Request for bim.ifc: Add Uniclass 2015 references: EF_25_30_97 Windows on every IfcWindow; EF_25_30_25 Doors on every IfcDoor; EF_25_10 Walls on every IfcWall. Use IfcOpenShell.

First a look at what the model holds.

```python
import ifcopenshell

model = ifcopenshell.open("bim.ifc")
print(model.schema)
print("classifications:", [c.Name for c in model.by_type("IfcClassification")])
for ifc_class in ("IfcDoor", "IfcRoof", "IfcStair", "IfcWall", "IfcWindow"):
    print(ifc_class, len(model.by_type(ifc_class)))
```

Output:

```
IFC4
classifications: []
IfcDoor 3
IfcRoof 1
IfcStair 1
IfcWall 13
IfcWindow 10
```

```python
import ifcopenshell
import ifcopenshell.api.classification

model = ifcopenshell.open("bim.ifc")

system = ifcopenshell.api.classification.add_classification(model, classification="Uniclass 2015")

codes = {
    "IfcWindow": ("EF_25_30_97", "Windows"),
    "IfcDoor": ("EF_25_30_25", "Doors"),
    "IfcWall": ("EF_25_10", "Walls"),
}
for ifc_class, (code, name) in codes.items():
    products = model.by_type(ifc_class)
    ifcopenshell.api.classification.add_reference(
        model, products=products, classification=system, identification=code, name=name
    )
    print(code, len(products))

model.write("bim_v2.ifc")
```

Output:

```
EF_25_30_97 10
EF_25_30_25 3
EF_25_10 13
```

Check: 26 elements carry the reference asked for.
